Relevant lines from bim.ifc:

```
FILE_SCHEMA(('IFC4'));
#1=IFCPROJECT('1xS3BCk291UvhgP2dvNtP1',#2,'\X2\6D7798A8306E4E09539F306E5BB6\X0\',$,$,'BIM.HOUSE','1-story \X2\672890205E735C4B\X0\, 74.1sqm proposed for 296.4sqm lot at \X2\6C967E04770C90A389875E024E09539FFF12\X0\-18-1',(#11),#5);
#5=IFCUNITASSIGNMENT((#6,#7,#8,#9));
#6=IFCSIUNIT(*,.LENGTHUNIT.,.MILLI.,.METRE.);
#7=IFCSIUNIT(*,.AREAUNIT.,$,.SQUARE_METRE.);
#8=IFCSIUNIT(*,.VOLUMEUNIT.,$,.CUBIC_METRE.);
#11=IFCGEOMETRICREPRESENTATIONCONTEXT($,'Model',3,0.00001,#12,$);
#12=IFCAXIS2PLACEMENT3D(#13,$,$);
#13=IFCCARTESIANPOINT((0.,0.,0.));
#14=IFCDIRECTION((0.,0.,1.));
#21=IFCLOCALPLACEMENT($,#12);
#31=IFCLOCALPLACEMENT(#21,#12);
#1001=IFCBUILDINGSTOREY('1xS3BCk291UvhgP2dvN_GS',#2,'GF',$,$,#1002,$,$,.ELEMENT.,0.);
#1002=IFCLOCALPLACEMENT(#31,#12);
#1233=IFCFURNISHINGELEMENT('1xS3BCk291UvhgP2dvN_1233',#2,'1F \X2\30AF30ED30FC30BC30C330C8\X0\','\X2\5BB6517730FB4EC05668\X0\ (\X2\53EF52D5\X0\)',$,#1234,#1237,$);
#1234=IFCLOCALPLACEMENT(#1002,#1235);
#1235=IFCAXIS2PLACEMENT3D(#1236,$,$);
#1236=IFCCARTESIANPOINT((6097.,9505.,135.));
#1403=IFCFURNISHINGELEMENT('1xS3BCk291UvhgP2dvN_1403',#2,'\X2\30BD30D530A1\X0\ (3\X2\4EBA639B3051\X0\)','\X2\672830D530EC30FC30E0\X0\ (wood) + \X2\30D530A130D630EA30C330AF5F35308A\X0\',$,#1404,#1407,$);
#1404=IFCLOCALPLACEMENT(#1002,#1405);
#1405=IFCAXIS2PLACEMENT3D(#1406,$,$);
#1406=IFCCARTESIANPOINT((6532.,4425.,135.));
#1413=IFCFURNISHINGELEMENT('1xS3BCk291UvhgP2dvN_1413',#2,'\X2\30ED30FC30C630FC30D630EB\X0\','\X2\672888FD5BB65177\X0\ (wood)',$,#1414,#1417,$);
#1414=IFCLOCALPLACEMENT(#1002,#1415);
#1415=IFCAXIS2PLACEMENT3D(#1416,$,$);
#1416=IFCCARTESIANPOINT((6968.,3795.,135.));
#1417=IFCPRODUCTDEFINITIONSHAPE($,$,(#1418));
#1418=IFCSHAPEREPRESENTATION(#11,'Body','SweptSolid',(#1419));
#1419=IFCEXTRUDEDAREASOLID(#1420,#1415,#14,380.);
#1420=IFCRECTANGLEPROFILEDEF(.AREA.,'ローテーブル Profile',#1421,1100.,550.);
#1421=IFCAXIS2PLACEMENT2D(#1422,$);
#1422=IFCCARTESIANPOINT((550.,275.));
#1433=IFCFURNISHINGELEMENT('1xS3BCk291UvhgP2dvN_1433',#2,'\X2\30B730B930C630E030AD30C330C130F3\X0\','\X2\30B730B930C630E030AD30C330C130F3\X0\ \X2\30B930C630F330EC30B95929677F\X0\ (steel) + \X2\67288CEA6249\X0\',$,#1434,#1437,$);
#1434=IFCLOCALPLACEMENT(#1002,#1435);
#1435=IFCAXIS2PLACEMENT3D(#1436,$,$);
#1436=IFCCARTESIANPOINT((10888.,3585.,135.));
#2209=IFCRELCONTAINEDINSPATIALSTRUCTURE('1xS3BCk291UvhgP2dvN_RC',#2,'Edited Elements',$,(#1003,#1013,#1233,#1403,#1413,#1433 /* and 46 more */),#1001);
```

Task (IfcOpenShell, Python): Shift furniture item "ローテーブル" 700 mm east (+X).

```python
import ifcopenshell
import ifcopenshell.api.geometry
import ifcopenshell.util.placement

model = ifcopenshell.open("bim.ifc")

item = model.by_id(1413)
matrix = ifcopenshell.util.placement.get_local_placement(item.ObjectPlacement)
matrix[0, 3] += 700.0
ifcopenshell.api.geometry.edit_object_placement(model, product=item, matrix=matrix, is_si=False)

print(ifcopenshell.util.placement.get_local_placement(item.ObjectPlacement).round(3) + 0.0)

model.write("bim_updated.ifc")
```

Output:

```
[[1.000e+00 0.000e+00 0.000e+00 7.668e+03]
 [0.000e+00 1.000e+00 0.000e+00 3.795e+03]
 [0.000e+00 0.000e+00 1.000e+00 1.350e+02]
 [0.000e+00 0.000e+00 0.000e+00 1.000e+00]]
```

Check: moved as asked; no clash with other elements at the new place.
